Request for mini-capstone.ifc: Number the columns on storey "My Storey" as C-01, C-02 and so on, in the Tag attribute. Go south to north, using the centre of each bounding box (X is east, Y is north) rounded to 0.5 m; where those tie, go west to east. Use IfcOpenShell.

First a look at what the model holds.

```python
import ifcopenshell
import ifcopenshell.util.element
import ifcopenshell.util.placement

model = ifcopenshell.open("mini-capstone.ifc")
print(model.schema)
storey = next(s for s in model.by_type("IfcBuildingStorey") if s.Name == "My Storey")
columns = [e for e in ifcopenshell.util.element.get_decomposition(storey) if e.is_a("IfcColumn")]
for e in sorted(columns, key=lambda e: e.id()):
    origin = ifcopenshell.util.placement.get_local_placement(e.ObjectPlacement)[:3, 3]
    print(e.id(), e.Tag, e.Name, origin.round(2) + 0.0, sep=" | ")
```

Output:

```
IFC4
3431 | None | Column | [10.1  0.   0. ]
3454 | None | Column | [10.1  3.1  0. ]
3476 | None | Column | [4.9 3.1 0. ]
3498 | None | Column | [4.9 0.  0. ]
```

```python
import ifcopenshell
import ifcopenshell.geom
import ifcopenshell.util.element
import ifcopenshell.util.shape

model = ifcopenshell.open("mini-capstone.ifc")
settings = ifcopenshell.geom.settings()
settings.set("use-world-coords", True)


def centre(element):
    shape = ifcopenshell.geom.create_shape(settings, element)
    return ifcopenshell.util.shape.get_bbox_centroid(shape.geometry)


storey = next(s for s in model.by_type("IfcBuildingStorey") if s.Name == "My Storey")
columns = [e for e in ifcopenshell.util.element.get_decomposition(storey) if e.is_a("IfcColumn")]

# Insertion points can sit at a corner or the storey origin, so sort by the geometry (in metres).
centres = {e: centre(e) for e in columns}
columns.sort(key=lambda e: (round(centres[e][1] / 0.5), centres[e][0]))

for i, e in enumerate(columns, start=1):
    number = f"C-{i:02d}"
    e.Tag = number
    print(e.id(), number)

model.write("mini-capstone_edited.ifc")
```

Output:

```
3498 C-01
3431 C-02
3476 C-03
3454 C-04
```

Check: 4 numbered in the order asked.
